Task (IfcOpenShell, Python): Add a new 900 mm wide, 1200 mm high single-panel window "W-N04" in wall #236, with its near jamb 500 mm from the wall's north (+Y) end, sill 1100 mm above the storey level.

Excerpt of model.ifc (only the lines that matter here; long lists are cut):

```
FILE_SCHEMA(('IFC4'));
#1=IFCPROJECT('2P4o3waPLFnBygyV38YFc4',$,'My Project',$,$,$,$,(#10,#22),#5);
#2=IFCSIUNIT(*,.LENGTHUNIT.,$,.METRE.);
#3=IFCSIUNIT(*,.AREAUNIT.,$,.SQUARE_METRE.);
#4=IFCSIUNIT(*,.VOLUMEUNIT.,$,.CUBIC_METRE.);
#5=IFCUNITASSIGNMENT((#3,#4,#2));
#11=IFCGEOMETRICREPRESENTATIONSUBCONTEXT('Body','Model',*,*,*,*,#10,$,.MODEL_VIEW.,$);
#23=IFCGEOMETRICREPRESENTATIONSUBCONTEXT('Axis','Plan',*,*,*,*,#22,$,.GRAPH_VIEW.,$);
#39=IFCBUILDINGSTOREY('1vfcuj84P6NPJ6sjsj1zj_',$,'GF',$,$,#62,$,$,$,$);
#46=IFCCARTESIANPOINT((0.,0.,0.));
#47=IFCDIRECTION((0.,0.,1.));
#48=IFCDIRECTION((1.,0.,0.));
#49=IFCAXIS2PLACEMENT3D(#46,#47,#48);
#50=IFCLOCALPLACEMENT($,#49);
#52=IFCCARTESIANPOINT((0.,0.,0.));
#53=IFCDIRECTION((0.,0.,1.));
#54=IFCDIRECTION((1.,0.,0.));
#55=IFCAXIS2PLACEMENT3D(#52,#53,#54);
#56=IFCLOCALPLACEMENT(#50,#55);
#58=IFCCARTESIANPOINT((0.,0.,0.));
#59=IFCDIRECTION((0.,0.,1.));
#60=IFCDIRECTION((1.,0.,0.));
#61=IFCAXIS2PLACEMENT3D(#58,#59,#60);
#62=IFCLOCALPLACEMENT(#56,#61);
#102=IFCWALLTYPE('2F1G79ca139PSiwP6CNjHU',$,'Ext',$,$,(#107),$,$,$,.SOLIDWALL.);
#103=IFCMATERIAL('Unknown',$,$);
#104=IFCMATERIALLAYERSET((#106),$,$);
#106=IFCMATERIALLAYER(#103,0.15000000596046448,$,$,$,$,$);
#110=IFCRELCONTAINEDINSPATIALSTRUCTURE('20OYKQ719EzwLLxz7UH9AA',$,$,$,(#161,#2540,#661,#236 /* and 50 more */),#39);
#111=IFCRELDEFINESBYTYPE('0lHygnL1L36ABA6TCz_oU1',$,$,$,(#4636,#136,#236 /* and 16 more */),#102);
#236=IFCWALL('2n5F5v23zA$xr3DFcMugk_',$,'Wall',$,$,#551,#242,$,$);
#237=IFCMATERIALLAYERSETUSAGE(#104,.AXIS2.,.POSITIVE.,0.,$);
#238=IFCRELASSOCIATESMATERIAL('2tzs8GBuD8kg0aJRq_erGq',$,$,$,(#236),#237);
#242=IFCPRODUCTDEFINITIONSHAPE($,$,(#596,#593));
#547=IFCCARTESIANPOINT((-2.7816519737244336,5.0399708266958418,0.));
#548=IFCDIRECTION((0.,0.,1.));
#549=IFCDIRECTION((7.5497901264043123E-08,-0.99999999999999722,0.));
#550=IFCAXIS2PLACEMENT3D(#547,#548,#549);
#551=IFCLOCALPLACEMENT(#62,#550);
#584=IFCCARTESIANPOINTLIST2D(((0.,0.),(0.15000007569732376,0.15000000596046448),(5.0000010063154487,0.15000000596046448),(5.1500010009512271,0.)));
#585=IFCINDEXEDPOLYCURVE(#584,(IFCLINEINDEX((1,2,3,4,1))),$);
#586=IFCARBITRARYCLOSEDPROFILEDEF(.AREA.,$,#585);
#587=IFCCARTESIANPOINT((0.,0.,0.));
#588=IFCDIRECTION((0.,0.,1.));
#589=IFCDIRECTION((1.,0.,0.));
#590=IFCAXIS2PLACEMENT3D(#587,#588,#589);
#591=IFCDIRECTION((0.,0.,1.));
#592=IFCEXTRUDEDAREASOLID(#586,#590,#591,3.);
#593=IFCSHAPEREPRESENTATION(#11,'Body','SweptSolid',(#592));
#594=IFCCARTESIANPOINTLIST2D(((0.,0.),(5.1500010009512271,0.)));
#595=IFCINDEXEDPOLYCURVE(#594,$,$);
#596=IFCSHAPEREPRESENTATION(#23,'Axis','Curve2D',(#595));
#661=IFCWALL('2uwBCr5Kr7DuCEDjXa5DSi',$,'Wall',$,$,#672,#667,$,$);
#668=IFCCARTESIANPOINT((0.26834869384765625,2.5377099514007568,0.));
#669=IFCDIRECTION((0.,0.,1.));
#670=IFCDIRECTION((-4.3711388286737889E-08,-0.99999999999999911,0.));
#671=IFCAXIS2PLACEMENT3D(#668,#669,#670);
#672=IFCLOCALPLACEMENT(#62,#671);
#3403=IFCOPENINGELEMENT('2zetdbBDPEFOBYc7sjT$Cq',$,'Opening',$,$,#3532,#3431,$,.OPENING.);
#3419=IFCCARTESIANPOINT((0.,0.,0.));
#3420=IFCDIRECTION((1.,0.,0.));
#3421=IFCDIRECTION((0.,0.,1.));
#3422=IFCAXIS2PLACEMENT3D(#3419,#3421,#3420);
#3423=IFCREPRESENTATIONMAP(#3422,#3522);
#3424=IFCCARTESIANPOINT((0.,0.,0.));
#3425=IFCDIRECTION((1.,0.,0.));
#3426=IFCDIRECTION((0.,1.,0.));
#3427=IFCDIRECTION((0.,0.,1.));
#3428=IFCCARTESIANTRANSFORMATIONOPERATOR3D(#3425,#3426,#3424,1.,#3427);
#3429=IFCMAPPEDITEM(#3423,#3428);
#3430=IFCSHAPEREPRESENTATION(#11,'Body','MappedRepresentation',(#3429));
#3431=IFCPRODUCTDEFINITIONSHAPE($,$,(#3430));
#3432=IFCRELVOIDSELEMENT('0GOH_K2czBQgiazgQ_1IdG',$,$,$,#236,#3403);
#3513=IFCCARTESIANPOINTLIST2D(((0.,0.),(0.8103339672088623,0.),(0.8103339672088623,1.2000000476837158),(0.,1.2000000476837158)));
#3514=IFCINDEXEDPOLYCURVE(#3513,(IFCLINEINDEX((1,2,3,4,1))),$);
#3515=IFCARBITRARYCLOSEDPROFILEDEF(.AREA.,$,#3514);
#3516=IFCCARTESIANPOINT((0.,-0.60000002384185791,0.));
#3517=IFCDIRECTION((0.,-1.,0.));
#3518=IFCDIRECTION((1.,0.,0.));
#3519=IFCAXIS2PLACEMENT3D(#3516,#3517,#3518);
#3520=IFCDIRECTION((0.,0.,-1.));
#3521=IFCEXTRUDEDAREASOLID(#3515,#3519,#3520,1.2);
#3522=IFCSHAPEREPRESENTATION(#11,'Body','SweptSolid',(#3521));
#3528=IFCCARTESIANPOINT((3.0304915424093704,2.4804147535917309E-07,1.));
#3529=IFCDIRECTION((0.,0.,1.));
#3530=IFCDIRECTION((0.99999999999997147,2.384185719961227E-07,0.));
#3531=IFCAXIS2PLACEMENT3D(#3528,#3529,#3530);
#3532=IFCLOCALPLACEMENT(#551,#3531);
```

```python
import numpy as np
import ifcopenshell
import ifcopenshell.api.feature
import ifcopenshell.api.geometry
import ifcopenshell.api.root
import ifcopenshell.api.spatial
import ifcopenshell.geom
import ifcopenshell.util.element
import ifcopenshell.util.placement
import ifcopenshell.util.representation
import ifcopenshell.util.shape
import ifcopenshell.util.unit

model = ifcopenshell.open("model.ifc")
unit_scale = ifcopenshell.util.unit.calculate_unit_scale(model)
settings = ifcopenshell.geom.settings()


def volume(element):
    """Net volume in cubic metres, openings subtracted."""
    shape = ifcopenshell.geom.create_shape(settings, element)
    return ifcopenshell.util.shape.get_volume(shape.geometry)


wall = model.by_guid("2n5F5v23zA$xr3DFcMugk_")
storey = ifcopenshell.util.element.get_container(wall, ifc_class="IfcBuildingStorey")
context = ifcopenshell.util.representation.get_context(model, "Model", "Body", "MODEL_VIEW")
before = volume(wall)

width, height, from_end, sill = 0.9, 1.2, 0.5, 1.1  # metres

# The wall runs along its own X axis, and the end named is its -X end.
wall_shape = ifcopenshell.geom.create_shape(settings, wall)
x, y, z = ifcopenshell.util.shape.get_vertices(wall_shape.geometry).T
start = x.min() + from_end
face, thickness = float(y.min()), float(y.max() - y.min())
wall_matrix = ifcopenshell.util.placement.get_local_placement(wall.ObjectPlacement)
level = ifcopenshell.util.placement.get_local_placement(storey.ObjectPlacement)[2, 3]


def in_wall(x, y):
    """Placement at x, y metres in the wall's axes, at sill height."""
    matrix = wall_matrix.copy()
    matrix[:, 3] = wall_matrix @ np.array([x / unit_scale, y / unit_scale, 0.0, 1.0])
    matrix[2, 3] = level + sill / unit_scale
    return matrix


# Opening: a box that overshoots both wall faces by 50 mm.
opening = ifcopenshell.api.root.create_entity(model, ifc_class="IfcOpeningElement", predefined_type="OPENING")
box = ifcopenshell.api.geometry.add_wall_representation(
    model, context=context, length=width, height=height, thickness=thickness + 0.1
)
ifcopenshell.api.geometry.assign_representation(model, product=opening, representation=box)
ifcopenshell.api.geometry.edit_object_placement(model, product=opening, matrix=in_wall(start, face - 0.05), is_si=False)
ifcopenshell.api.feature.add_feature(model, feature=opening, element=wall)

window = ifcopenshell.api.root.create_entity(model, ifc_class="IfcWindow", name="W-N04", predefined_type="WINDOW")
window.OverallWidth, window.OverallHeight = width / unit_scale, height / unit_scale
window.PartitioningType = "SINGLE_PANEL"
body = ifcopenshell.api.geometry.add_window_representation(
    model,
    context=context,
    overall_width=window.OverallWidth,
    overall_height=window.OverallHeight,
    partition_type="SINGLE_PANEL",
)
ifcopenshell.api.geometry.assign_representation(model, product=window, representation=body)
ifcopenshell.api.spatial.assign_container(model, products=[window], relating_structure=storey)
ifcopenshell.api.feature.add_filling(model, opening=opening, element=window)

# Centre the window in the wall's thickness.
ifcopenshell.api.geometry.edit_object_placement(model, product=window, matrix=in_wall(start, face), is_si=False)
window_shape = ifcopenshell.geom.create_shape(settings, window)
depth = ifcopenshell.util.shape.get_vertices(window_shape.geometry)[:, 1]
offset = face + thickness / 2 - (depth.min() + depth.max()) / 2
ifcopenshell.api.geometry.edit_object_placement(model, product=window, matrix=in_wall(start, offset), is_si=False)

after = volume(wall)

print(f"wall volume {before:.3f} -> {after:.3f} m3")

model.write("model_edited.ifc")
```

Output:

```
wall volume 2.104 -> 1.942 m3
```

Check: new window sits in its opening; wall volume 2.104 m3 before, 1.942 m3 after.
